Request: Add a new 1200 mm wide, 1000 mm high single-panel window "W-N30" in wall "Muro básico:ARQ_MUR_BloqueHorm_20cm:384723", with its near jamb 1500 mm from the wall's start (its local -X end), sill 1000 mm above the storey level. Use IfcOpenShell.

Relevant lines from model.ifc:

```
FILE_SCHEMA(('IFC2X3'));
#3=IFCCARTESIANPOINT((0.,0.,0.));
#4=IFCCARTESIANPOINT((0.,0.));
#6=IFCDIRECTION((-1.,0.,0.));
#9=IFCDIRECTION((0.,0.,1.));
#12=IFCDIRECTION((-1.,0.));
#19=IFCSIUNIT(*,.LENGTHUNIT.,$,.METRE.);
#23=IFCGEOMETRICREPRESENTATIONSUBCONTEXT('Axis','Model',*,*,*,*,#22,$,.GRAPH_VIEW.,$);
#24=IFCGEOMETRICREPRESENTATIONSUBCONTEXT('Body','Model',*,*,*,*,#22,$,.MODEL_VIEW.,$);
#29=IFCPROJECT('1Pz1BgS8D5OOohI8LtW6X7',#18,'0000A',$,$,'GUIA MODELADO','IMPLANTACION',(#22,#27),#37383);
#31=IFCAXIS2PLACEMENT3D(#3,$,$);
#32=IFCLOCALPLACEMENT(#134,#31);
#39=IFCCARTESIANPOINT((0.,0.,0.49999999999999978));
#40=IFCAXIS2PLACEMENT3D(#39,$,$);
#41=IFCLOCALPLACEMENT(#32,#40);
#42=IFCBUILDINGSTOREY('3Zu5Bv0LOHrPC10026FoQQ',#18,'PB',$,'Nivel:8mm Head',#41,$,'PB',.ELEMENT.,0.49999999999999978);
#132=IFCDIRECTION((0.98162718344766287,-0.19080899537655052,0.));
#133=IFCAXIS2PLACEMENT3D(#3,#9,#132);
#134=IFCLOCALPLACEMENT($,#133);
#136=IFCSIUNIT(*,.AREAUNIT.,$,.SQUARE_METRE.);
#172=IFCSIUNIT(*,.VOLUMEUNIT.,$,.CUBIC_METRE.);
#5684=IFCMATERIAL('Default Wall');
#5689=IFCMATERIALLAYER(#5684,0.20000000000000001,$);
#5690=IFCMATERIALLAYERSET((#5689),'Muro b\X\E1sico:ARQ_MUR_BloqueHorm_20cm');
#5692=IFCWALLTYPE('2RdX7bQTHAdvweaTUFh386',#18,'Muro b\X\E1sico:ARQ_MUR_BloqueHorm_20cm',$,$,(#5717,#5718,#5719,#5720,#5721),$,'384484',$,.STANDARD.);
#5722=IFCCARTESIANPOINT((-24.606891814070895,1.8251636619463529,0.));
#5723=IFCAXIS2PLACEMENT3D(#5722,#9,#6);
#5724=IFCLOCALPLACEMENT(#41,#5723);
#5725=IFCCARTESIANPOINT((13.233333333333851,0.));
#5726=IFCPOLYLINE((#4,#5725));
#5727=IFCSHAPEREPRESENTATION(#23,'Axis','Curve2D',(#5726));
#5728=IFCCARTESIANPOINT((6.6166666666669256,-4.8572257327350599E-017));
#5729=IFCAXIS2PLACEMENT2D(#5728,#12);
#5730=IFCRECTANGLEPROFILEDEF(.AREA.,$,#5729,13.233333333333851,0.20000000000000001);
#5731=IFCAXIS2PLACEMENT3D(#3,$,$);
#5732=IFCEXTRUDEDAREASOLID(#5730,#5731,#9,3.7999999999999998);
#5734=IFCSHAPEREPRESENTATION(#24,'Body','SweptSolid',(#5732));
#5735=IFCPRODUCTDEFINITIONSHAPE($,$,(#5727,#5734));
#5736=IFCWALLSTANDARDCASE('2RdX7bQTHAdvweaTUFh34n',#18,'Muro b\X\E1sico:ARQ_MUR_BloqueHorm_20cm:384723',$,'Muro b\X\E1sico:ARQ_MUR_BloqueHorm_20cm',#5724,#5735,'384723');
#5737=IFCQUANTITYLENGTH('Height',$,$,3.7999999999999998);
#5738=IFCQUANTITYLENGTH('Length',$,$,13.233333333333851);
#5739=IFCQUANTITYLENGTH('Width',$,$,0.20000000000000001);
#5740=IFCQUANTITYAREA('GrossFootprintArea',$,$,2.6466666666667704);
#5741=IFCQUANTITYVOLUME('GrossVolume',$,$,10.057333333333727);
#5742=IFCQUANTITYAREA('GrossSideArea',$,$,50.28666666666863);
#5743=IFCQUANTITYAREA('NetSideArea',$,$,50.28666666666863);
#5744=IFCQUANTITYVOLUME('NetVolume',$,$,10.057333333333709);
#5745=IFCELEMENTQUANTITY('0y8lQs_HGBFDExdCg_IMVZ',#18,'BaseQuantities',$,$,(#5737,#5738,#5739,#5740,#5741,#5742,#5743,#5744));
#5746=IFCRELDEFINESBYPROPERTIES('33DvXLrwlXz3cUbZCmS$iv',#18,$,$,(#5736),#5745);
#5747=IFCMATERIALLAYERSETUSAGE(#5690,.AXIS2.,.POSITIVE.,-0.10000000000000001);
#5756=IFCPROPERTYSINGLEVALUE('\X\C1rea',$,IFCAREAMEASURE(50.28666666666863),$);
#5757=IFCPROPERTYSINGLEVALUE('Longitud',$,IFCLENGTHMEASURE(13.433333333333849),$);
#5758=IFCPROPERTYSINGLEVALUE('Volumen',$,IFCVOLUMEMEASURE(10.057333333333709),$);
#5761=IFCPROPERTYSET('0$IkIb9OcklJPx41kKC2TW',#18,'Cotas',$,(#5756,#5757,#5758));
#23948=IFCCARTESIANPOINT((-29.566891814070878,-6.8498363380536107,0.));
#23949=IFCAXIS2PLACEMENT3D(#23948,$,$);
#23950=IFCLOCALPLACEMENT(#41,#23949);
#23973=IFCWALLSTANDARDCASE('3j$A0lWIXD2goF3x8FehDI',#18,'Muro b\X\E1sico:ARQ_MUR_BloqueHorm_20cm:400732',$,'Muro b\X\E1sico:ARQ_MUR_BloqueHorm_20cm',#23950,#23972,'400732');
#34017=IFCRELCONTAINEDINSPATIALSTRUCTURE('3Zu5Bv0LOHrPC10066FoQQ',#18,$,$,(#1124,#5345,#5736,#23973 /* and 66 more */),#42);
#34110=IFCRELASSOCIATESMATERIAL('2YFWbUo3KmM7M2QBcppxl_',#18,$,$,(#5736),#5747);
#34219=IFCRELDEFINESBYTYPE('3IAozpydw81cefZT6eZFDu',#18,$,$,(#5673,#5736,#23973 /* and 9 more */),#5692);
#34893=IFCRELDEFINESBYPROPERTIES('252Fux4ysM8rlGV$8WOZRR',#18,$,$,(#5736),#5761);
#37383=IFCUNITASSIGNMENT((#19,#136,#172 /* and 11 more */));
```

```python
import numpy as np
import ifcopenshell
import ifcopenshell.api.feature
import ifcopenshell.api.geometry
import ifcopenshell.api.pset
import ifcopenshell.api.root
import ifcopenshell.api.spatial
import ifcopenshell.api.type
import ifcopenshell.geom
import ifcopenshell.util.element
import ifcopenshell.util.placement
import ifcopenshell.util.representation
import ifcopenshell.util.shape
import ifcopenshell.util.unit

model = ifcopenshell.open("model.ifc")
unit_scale = ifcopenshell.util.unit.calculate_unit_scale(model)
area_scale = ifcopenshell.util.unit.calculate_unit_scale(model, "AREAUNIT")
volume_scale = ifcopenshell.util.unit.calculate_unit_scale(model, "VOLUMEUNIT")
settings = ifcopenshell.geom.settings()


def volume(element):
    """Net volume in cubic metres, openings subtracted."""
    shape = ifcopenshell.geom.create_shape(settings, element)
    return ifcopenshell.util.shape.get_volume(shape.geometry)


wall = model.by_guid("2RdX7bQTHAdvweaTUFh34n")
storey = ifcopenshell.util.element.get_container(wall, ifc_class="IfcBuildingStorey")
context = ifcopenshell.util.representation.get_context(model, "Model", "Body", "MODEL_VIEW")
before = volume(wall)

width, height, from_end, sill = 1.2, 1, 1.5, 1  # metres

# The wall runs along its own X axis, and the end named is its -X end.
wall_shape = ifcopenshell.geom.create_shape(settings, wall)
x, y, z = ifcopenshell.util.shape.get_vertices(wall_shape.geometry).T
start = x.min() + from_end
face, thickness = float(y.min()), float(y.max() - y.min())
wall_matrix = ifcopenshell.util.placement.get_local_placement(wall.ObjectPlacement)
level = ifcopenshell.util.placement.get_local_placement(storey.ObjectPlacement)[2, 3]


def in_wall(x, y):
    """Placement at x, y metres in the wall's axes, at sill height."""
    matrix = wall_matrix.copy()
    matrix[:, 3] = wall_matrix @ np.array([x / unit_scale, y / unit_scale, 0.0, 1.0])
    matrix[2, 3] = level + sill / unit_scale
    return matrix


# Opening: a box that overshoots both wall faces by 50 mm.
opening = ifcopenshell.api.root.create_entity(model, ifc_class="IfcOpeningElement")
box = ifcopenshell.api.geometry.add_wall_representation(
    model, context=context, length=width, height=height, thickness=thickness + 0.1
)
ifcopenshell.api.geometry.assign_representation(model, product=opening, representation=box)
ifcopenshell.api.geometry.edit_object_placement(model, product=opening, matrix=in_wall(start, face - 0.05), is_si=False)
ifcopenshell.api.feature.add_feature(model, feature=opening, element=wall)

window = ifcopenshell.api.root.create_entity(model, ifc_class="IfcWindow", name="W-N30")
window.OverallWidth, window.OverallHeight = width / unit_scale, height / unit_scale
body = ifcopenshell.api.geometry.add_window_representation(
    model,
    context=context,
    overall_width=window.OverallWidth,
    overall_height=window.OverallHeight,
    partition_type="SINGLE_PANEL",
)
ifcopenshell.api.geometry.assign_representation(model, product=window, representation=body)
ifcopenshell.api.spatial.assign_container(model, products=[window], relating_structure=storey)
fills = ifcopenshell.api.feature.add_filling(model, opening=opening, element=window)
fills.OwnerHistory = window.OwnerHistory  # required in IFC2X3

# IFC2X3 keeps the operation on the window style.
style = ifcopenshell.api.root.create_entity(model, ifc_class="IfcWindowStyle", name="W-N30")
style.OperationType, style.ConstructionType = "SINGLE_PANEL", "NOTDEFINED"
style.ParameterTakesPrecedence = style.Sizeable = False
ifcopenshell.api.type.assign_type(model, related_objects=[window], relating_type=style)

# Centre the window in the wall's thickness.
ifcopenshell.api.geometry.edit_object_placement(model, product=window, matrix=in_wall(start, face), is_si=False)
window_shape = ifcopenshell.geom.create_shape(settings, window)
depth = ifcopenshell.util.shape.get_vertices(window_shape.geometry)[:, 1]
offset = face + thickness / 2 - (depth.min() + depth.max()) / 2
ifcopenshell.api.geometry.edit_object_placement(model, product=window, matrix=in_wall(start, offset), is_si=False)

after = volume(wall)

# Update the wall's stored quantities.
qto = model.by_id(ifcopenshell.util.element.get_pset(wall, "BaseQuantities", should_inherit=False)["id"])
ifcopenshell.api.pset.edit_qto(model, qto=qto, properties={
    "NetSideArea": after / thickness / area_scale,
    "NetVolume": after / volume_scale,
})
pset = model.by_id(ifcopenshell.util.element.get_pset(wall, "Cotas", should_inherit=False)["id"])
ifcopenshell.api.pset.edit_pset(model, pset=pset, properties={
    "Área": model.create_entity("IfcAreaMeasure", after / thickness / area_scale),
    "Volumen": model.create_entity("IfcVolumeMeasure", after / volume_scale),
})

print(f"wall volume {before:.3f} -> {after:.3f} m3")

model.write("model_v2.ifc")
```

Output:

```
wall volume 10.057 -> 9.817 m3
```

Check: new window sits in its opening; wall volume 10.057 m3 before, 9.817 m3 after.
